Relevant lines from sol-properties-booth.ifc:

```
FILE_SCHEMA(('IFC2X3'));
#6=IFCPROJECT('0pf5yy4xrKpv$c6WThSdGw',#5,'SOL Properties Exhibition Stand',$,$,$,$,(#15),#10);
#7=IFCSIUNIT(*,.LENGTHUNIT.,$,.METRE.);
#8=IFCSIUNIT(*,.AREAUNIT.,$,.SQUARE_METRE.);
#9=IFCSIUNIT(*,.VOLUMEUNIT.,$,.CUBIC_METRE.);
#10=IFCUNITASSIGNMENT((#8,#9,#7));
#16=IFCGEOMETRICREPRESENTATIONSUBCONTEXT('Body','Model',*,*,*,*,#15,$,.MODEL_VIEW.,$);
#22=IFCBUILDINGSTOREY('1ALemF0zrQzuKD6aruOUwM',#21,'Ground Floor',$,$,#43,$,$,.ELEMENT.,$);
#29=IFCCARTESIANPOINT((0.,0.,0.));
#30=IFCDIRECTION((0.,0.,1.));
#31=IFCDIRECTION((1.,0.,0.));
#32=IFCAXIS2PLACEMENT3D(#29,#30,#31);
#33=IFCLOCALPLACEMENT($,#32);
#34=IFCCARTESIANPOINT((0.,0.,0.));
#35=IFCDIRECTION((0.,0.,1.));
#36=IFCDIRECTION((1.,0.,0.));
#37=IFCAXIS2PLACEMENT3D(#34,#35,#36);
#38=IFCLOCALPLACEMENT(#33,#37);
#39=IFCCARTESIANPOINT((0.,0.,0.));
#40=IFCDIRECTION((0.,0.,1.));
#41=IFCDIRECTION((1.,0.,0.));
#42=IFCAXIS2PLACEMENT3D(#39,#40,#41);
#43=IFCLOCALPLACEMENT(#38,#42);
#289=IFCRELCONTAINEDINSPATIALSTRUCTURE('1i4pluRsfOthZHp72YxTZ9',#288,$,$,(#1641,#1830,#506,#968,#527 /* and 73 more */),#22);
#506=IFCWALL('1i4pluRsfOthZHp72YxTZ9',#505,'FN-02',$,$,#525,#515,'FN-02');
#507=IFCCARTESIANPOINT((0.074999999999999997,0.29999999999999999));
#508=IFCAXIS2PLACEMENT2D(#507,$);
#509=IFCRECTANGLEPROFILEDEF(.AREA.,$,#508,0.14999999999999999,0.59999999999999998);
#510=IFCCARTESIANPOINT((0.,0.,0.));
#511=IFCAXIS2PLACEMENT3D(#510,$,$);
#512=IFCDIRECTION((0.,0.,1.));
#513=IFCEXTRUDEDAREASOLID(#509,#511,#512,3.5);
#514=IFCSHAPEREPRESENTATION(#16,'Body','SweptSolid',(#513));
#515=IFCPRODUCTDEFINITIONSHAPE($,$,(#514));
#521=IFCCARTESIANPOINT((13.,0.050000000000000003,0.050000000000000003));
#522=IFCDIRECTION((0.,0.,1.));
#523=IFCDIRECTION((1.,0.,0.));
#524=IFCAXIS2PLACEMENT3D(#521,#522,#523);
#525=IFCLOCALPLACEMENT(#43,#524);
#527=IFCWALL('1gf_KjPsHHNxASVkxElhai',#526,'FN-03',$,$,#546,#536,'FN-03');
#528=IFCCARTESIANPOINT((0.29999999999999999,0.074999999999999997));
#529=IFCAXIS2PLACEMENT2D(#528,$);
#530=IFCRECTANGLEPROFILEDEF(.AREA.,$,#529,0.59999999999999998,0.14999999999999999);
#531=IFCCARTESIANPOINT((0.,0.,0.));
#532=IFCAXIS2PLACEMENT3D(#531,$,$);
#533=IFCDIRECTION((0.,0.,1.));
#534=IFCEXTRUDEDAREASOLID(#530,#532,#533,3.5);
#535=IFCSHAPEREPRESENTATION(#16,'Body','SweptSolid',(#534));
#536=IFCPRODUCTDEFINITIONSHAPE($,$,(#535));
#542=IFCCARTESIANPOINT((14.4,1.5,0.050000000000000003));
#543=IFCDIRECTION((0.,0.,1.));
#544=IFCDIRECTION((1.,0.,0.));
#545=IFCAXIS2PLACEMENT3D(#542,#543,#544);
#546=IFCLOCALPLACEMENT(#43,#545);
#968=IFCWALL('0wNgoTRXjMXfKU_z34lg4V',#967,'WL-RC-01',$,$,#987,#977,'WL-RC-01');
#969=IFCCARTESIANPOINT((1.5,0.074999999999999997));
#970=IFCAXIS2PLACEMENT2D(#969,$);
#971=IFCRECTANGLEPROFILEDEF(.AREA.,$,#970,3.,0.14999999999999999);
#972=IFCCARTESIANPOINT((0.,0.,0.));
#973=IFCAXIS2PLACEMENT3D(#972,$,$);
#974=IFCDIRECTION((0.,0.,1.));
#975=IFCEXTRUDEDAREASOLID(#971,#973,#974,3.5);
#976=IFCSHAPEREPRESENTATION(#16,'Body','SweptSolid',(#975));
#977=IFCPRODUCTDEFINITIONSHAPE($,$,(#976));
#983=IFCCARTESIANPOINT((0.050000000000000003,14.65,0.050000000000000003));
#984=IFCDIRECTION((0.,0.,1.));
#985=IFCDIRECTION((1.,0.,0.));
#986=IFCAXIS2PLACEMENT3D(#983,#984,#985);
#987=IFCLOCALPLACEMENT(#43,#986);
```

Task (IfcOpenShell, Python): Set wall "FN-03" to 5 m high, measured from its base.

```python
import ifcopenshell
import ifcopenshell.geom
import ifcopenshell.util.representation
import ifcopenshell.util.shape

model = ifcopenshell.open("sol-properties-booth.ifc")
settings = ifcopenshell.geom.settings()


def volume(element):
    """Net volume in cubic metres, openings subtracted."""
    shape = ifcopenshell.geom.create_shape(settings, element)
    return ifcopenshell.util.shape.get_volume(shape.geometry)


wall = model.by_id(527)
before = volume(wall)

body = ifcopenshell.util.representation.get_representation(wall, "Model", "Body")
solid = body.Items[0]
old_height = solid.Depth
solid.Depth = 5.0
after = volume(wall)

print(f"height {old_height:g} -> {solid.Depth:g}, volume {before:.3f} -> {after:.3f} m3")

model.write("sol-properties-booth_updated.ifc")
```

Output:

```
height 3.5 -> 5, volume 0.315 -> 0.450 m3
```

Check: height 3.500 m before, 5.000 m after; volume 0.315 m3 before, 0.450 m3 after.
